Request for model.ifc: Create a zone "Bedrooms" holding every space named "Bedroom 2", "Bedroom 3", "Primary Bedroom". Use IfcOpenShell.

First a look at what the model holds.

```python
import ifcopenshell

model = ifcopenshell.open("model.ifc")
print(model.schema)
seen = {}
for space in model.by_type("IfcSpace"):
    seen[space.LongName] = seen.get(space.LongName, 0) + 1
for name, count in sorted(seen.items(), key=str):
    print(count, "x", name)
print("zones:", [z.Name for z in model.by_type("IfcZone")][:20])
```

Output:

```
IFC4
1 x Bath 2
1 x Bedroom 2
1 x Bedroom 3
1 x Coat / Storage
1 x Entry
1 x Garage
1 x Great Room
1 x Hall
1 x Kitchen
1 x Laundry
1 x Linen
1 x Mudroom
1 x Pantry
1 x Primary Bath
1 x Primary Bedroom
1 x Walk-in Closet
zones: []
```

```python
import ifcopenshell
import ifcopenshell.api.group
import ifcopenshell.api.root

model = ifcopenshell.open("model.ifc")

names = {"Bedroom 2", "Bedroom 3", "Primary Bedroom"}
spaces = [s for s in model.by_type("IfcSpace") if s.LongName in names]

zone = ifcopenshell.api.root.create_entity(model, ifc_class="IfcZone", name="Bedrooms")
ifcopenshell.api.group.assign_group(model, products=spaces, group=zone)
print(len(spaces), "spaces in", zone.Name)

model.write("model_edited.ifc")
```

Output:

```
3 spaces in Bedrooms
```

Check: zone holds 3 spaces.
